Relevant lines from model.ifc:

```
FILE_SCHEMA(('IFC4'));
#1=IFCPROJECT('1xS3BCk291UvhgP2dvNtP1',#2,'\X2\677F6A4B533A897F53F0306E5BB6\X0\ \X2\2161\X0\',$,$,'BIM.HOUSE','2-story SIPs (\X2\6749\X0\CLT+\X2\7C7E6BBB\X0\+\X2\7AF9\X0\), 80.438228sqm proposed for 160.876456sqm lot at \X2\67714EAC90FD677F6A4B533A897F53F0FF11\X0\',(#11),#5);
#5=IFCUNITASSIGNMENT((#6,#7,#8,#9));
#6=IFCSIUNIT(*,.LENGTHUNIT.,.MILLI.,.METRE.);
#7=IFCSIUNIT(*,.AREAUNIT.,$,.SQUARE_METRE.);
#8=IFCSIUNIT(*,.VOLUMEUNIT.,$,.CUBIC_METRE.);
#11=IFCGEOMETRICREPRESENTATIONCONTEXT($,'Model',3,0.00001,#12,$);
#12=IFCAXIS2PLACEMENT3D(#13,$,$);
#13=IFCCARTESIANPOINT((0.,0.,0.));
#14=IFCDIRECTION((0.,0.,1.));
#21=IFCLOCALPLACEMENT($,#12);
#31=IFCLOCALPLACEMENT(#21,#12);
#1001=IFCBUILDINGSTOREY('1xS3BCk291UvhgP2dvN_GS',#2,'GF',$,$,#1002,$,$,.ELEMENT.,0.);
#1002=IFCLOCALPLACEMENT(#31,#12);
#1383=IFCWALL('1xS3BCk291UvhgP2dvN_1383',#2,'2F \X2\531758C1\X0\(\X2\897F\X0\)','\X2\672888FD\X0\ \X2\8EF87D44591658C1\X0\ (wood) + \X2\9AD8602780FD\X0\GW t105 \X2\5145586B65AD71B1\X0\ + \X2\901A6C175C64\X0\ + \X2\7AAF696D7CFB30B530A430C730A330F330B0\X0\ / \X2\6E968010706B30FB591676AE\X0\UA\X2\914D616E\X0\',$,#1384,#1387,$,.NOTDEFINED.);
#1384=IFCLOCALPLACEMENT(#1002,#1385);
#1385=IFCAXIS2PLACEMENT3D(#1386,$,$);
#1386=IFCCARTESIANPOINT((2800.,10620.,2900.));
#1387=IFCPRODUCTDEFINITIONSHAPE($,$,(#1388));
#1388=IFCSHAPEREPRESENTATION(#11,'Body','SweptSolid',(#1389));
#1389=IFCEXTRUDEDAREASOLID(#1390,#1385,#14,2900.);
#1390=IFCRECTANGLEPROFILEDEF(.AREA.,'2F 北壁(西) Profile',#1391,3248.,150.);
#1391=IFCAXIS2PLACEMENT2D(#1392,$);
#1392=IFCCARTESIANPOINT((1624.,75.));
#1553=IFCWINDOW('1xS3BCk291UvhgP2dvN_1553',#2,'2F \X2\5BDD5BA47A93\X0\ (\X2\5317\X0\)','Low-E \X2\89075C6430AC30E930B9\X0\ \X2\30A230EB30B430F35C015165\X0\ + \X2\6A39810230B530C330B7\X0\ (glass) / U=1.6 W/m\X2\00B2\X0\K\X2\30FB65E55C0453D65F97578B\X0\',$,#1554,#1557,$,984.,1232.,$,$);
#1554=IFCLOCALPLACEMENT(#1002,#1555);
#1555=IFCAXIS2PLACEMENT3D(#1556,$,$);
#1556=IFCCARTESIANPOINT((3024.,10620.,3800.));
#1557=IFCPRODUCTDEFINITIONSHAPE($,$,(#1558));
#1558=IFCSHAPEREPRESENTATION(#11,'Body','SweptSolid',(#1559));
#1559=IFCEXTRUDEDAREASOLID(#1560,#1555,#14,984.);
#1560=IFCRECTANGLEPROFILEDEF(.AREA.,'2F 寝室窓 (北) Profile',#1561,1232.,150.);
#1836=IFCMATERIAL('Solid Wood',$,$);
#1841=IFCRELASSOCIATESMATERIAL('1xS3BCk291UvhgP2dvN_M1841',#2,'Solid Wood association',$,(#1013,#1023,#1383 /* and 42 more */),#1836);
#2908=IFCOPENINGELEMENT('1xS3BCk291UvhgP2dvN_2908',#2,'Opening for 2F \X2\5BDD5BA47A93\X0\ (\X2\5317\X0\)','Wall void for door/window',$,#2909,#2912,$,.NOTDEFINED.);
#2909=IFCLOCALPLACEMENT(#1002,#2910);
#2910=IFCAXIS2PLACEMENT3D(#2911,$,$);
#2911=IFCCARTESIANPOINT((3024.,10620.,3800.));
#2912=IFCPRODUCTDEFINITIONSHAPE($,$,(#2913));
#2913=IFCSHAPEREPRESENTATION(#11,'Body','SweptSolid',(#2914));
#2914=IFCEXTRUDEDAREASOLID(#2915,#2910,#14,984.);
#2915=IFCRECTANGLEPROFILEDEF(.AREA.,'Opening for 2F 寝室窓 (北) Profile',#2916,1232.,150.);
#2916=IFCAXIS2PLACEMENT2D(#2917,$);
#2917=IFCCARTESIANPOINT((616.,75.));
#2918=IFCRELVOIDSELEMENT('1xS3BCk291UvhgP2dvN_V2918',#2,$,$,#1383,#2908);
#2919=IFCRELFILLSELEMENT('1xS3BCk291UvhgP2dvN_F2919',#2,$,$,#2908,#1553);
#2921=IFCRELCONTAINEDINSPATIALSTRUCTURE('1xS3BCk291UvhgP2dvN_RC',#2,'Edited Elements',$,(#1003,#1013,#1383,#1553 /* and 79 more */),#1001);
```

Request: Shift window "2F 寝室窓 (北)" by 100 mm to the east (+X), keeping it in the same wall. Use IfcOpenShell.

```python
import ifcopenshell
import ifcopenshell.api.geometry
import ifcopenshell.util.placement

model = ifcopenshell.open("model.ifc")

window = model.by_id(1553)
opening = window.FillsVoids[0].RelatingOpeningElement
wall = opening.VoidsElements[0].RelatingBuildingElement

wall_matrix = ifcopenshell.util.placement.get_local_placement(wall.ObjectPlacement)
shift = wall_matrix[:3, 0] * 100.0
before = ifcopenshell.util.placement.get_local_placement(window.ObjectPlacement)[:3, 3].copy()

# The window is not placed relative to its opening, so move both.
for product in (opening, window):
    matrix = ifcopenshell.util.placement.get_local_placement(product.ObjectPlacement)
    matrix[:3, 3] += shift
    ifcopenshell.api.geometry.edit_object_placement(model, product=product, matrix=matrix, is_si=False)

after = ifcopenshell.util.placement.get_local_placement(window.ObjectPlacement)[:3, 3]
print("window moved by", (after - before).round(3) + 0.0)

model.write("model_updated.ifc")
```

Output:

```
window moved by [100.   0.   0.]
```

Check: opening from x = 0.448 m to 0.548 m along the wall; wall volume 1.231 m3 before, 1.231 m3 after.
